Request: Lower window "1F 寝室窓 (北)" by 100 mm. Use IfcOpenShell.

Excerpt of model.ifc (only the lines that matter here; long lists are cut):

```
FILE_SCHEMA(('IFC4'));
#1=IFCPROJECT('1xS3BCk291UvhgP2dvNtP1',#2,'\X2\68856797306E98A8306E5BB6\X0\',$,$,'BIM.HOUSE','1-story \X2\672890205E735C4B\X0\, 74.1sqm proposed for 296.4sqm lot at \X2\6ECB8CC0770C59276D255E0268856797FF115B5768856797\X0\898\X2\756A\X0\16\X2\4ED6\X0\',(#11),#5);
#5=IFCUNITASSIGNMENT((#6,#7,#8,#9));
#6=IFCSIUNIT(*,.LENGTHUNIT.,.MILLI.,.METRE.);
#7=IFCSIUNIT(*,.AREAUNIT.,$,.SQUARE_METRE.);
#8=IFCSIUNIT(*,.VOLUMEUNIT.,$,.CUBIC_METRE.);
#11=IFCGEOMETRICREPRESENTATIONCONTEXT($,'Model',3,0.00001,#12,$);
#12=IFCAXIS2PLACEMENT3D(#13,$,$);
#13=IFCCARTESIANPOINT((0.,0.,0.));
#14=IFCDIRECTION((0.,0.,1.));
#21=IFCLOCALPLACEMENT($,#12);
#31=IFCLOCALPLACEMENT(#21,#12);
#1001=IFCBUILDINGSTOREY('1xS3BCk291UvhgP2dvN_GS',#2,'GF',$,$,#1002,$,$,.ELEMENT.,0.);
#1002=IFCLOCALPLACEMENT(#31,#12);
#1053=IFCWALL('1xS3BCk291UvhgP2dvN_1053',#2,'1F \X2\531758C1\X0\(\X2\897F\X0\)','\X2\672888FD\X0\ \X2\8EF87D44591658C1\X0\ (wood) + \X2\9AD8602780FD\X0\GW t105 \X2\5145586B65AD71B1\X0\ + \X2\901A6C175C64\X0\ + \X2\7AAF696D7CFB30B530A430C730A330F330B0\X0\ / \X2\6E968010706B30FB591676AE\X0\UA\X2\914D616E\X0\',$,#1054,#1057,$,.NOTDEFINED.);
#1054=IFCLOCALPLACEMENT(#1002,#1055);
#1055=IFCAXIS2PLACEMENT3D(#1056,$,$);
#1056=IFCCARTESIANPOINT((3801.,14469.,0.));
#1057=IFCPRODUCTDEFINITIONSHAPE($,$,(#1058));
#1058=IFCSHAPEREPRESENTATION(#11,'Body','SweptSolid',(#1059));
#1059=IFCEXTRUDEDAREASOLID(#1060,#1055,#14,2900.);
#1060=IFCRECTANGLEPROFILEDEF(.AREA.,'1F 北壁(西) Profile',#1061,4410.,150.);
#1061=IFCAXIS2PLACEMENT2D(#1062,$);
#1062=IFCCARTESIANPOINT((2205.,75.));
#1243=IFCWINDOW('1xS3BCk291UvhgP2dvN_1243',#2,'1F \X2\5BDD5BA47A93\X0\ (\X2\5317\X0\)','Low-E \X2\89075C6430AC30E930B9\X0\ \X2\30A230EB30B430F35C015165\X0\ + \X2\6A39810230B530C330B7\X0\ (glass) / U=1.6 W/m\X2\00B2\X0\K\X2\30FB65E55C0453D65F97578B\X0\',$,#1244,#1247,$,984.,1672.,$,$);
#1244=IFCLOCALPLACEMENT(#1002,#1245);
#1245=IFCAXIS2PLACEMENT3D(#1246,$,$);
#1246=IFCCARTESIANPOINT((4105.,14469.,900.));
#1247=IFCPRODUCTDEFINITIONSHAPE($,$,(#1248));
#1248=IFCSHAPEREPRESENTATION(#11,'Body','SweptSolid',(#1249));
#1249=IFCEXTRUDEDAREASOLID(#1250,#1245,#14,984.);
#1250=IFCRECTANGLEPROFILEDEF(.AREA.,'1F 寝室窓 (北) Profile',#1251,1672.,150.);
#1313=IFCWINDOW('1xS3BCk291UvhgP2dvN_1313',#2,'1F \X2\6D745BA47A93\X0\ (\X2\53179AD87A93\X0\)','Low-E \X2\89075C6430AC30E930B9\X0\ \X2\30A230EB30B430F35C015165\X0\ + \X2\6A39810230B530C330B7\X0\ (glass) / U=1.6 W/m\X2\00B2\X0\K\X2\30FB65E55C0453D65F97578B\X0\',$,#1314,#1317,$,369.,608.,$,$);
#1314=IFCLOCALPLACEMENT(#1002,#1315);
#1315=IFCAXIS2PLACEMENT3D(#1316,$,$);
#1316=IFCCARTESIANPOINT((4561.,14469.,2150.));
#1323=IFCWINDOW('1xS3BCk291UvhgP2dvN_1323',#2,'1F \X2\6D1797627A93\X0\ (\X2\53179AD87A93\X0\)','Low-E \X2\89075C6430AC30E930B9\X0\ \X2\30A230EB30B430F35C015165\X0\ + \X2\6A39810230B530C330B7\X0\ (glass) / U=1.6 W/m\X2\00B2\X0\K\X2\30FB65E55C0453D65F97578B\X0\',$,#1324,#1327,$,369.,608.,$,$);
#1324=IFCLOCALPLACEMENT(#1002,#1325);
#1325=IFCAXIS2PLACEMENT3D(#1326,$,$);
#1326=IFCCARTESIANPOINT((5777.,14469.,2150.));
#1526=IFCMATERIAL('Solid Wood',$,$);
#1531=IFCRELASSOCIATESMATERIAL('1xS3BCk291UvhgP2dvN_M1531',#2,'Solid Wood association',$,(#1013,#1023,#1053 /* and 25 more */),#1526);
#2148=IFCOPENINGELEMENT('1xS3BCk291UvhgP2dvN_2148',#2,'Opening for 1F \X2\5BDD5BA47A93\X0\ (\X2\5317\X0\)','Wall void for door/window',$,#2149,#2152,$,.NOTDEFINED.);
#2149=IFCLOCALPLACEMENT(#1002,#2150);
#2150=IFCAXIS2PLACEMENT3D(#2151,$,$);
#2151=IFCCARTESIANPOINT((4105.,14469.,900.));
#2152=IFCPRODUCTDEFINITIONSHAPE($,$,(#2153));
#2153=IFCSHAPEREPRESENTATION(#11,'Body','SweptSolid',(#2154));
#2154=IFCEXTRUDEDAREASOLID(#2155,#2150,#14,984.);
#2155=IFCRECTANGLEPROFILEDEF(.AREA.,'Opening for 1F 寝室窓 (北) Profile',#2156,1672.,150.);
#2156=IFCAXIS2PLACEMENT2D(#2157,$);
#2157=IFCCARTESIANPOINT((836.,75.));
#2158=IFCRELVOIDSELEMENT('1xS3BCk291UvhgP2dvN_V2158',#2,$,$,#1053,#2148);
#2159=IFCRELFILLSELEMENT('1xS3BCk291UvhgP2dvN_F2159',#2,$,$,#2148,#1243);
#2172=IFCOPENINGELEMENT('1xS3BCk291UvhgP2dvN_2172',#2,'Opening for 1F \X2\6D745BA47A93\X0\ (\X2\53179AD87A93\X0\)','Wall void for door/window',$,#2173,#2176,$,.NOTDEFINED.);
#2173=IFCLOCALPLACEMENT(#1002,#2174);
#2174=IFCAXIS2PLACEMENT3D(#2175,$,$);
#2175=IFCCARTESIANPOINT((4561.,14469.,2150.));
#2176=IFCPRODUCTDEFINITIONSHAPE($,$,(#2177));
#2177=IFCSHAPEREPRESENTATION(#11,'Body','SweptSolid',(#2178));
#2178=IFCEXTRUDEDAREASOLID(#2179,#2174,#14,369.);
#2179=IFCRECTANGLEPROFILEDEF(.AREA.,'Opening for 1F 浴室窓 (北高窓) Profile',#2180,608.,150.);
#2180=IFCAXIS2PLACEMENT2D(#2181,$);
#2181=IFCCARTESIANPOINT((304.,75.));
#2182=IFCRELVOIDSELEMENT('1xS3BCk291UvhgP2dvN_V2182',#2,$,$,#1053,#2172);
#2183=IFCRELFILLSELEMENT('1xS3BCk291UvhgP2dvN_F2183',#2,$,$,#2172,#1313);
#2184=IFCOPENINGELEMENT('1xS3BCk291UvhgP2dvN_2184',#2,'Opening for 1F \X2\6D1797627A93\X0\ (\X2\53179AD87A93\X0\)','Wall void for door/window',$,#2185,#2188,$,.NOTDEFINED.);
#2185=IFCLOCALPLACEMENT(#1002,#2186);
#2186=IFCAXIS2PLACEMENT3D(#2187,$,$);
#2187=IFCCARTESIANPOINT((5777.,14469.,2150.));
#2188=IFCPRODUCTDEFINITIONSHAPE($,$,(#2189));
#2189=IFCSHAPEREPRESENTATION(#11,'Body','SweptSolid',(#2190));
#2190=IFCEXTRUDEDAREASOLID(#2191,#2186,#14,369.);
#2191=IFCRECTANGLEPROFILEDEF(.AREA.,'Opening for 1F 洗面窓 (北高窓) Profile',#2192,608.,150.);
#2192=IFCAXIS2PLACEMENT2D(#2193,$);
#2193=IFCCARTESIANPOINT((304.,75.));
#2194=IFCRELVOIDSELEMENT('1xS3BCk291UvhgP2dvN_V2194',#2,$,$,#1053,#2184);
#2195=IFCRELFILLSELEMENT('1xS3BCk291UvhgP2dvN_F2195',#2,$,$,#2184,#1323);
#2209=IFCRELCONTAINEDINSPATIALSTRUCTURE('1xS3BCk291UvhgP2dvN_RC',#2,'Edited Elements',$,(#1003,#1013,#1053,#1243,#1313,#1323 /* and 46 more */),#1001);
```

```python
import numpy as np
import ifcopenshell
import ifcopenshell.api.geometry
import ifcopenshell.util.placement
import ifcopenshell.util.unit

model = ifcopenshell.open("model.ifc")
unit_scale = ifcopenshell.util.unit.calculate_unit_scale(model)

window = model.by_guid("1xS3BCk291UvhgP2dvN_1243")
opening = window.FillsVoids[0].RelatingOpeningElement
dz = -0.1 / unit_scale

shift = np.array([0.0, 0.0, dz])
# The window is not placed relative to its opening, so move both.
for product in (opening, window):
    matrix = ifcopenshell.util.placement.get_local_placement(product.ObjectPlacement)
    matrix[:3, 3] += shift
    ifcopenshell.api.geometry.edit_object_placement(model, product=product, matrix=matrix, is_si=False)

print(f"moved by {dz * unit_scale:+.3f} m")

model.write("model_rev.ifc")
```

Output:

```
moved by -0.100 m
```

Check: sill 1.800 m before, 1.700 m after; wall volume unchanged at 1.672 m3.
